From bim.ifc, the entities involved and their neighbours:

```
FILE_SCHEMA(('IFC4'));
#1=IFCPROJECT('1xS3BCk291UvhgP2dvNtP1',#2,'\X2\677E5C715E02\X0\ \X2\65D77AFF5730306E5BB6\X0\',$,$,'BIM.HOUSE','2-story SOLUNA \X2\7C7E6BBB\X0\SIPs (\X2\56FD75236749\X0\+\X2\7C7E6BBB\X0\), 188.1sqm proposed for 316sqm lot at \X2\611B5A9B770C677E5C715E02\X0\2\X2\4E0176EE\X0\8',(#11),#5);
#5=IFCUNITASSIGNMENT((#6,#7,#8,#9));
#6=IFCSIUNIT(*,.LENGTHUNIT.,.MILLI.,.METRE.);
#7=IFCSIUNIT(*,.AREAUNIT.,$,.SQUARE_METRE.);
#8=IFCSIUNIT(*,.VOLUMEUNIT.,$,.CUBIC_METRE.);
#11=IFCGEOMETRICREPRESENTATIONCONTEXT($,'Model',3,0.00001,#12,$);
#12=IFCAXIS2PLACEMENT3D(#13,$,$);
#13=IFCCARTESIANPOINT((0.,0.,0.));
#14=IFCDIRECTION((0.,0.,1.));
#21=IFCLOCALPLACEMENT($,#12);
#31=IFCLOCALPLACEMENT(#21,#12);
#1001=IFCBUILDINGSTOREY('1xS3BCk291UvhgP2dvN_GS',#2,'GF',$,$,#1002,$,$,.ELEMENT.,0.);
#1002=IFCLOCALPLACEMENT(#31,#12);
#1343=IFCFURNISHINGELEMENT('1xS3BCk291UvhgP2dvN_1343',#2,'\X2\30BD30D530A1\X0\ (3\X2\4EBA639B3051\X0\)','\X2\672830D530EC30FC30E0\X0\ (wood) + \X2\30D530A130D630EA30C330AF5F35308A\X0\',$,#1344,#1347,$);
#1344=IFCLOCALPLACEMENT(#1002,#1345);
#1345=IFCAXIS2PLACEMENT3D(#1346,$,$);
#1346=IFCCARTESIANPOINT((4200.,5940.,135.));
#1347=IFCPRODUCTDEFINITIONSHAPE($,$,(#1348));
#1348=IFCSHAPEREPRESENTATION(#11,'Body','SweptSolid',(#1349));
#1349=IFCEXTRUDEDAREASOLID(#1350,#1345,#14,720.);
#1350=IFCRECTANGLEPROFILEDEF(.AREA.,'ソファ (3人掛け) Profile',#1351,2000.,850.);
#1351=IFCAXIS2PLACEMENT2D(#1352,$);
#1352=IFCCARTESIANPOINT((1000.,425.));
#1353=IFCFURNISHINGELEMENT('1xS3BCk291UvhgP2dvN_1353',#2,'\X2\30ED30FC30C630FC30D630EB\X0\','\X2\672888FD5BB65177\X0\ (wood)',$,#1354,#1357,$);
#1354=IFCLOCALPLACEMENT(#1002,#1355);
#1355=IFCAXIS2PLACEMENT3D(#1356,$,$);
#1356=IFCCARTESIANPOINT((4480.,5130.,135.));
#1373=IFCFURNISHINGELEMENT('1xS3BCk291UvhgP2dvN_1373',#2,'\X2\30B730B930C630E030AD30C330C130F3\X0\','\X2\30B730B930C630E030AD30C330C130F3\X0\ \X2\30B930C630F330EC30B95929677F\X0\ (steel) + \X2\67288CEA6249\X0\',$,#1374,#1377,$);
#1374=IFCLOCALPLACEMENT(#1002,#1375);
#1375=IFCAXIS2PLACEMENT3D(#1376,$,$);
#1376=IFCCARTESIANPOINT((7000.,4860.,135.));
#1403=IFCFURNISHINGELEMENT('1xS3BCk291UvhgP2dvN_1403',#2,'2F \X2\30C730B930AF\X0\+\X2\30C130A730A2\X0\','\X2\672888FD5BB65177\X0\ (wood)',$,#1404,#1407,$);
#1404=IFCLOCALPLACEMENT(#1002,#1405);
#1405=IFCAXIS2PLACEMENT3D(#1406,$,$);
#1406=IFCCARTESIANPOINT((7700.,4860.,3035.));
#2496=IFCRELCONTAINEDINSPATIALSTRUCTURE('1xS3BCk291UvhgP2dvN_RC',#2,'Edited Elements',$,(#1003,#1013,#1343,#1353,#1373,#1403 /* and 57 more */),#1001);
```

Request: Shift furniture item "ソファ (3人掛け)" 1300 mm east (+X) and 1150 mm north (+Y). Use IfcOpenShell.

```python
import ifcopenshell
import ifcopenshell.api.geometry
import ifcopenshell.util.placement
import ifcopenshell.util.unit

model = ifcopenshell.open("bim.ifc")
unit_scale = ifcopenshell.util.unit.calculate_unit_scale(model)

item = model.by_guid("1xS3BCk291UvhgP2dvN_1343")
matrix = ifcopenshell.util.placement.get_local_placement(item.ObjectPlacement)
matrix[0, 3] += 1.3 / unit_scale
matrix[1, 3] += 1.15 / unit_scale
ifcopenshell.api.geometry.edit_object_placement(model, product=item, matrix=matrix, is_si=False)

print(ifcopenshell.util.placement.get_local_placement(item.ObjectPlacement).round(3) + 0.0)

model.write("bim_v2.ifc")
```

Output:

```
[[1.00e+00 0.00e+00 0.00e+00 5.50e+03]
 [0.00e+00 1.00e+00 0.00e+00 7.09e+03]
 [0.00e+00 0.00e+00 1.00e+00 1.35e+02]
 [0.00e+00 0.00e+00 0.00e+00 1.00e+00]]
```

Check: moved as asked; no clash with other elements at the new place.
